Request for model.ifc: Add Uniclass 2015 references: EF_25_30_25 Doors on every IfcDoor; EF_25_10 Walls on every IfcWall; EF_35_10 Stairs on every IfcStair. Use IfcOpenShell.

First a look at what the model holds.

```python
import ifcopenshell

model = ifcopenshell.open("model.ifc")
print(model.schema)
print("classifications:", [c.Name for c in model.by_type("IfcClassification")])
for ifc_class in ("IfcDoor", "IfcRoof", "IfcStair", "IfcWall", "IfcWindow"):
    print(ifc_class, len(model.by_type(ifc_class)))
```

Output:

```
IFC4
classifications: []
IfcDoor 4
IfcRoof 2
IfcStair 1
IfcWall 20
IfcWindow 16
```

```python
import ifcopenshell
import ifcopenshell.api.classification

model = ifcopenshell.open("model.ifc")

system = ifcopenshell.api.classification.add_classification(model, classification="Uniclass 2015")

codes = {
    "IfcDoor": ("EF_25_30_25", "Doors"),
    "IfcWall": ("EF_25_10", "Walls"),
    "IfcStair": ("EF_35_10", "Stairs"),
}
for ifc_class, (code, name) in codes.items():
    products = model.by_type(ifc_class)
    ifcopenshell.api.classification.add_reference(
        model, products=products, classification=system, identification=code, name=name
    )
    print(code, len(products))

model.write("model_rev.ifc")
```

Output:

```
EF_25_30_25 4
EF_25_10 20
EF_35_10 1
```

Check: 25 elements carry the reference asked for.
